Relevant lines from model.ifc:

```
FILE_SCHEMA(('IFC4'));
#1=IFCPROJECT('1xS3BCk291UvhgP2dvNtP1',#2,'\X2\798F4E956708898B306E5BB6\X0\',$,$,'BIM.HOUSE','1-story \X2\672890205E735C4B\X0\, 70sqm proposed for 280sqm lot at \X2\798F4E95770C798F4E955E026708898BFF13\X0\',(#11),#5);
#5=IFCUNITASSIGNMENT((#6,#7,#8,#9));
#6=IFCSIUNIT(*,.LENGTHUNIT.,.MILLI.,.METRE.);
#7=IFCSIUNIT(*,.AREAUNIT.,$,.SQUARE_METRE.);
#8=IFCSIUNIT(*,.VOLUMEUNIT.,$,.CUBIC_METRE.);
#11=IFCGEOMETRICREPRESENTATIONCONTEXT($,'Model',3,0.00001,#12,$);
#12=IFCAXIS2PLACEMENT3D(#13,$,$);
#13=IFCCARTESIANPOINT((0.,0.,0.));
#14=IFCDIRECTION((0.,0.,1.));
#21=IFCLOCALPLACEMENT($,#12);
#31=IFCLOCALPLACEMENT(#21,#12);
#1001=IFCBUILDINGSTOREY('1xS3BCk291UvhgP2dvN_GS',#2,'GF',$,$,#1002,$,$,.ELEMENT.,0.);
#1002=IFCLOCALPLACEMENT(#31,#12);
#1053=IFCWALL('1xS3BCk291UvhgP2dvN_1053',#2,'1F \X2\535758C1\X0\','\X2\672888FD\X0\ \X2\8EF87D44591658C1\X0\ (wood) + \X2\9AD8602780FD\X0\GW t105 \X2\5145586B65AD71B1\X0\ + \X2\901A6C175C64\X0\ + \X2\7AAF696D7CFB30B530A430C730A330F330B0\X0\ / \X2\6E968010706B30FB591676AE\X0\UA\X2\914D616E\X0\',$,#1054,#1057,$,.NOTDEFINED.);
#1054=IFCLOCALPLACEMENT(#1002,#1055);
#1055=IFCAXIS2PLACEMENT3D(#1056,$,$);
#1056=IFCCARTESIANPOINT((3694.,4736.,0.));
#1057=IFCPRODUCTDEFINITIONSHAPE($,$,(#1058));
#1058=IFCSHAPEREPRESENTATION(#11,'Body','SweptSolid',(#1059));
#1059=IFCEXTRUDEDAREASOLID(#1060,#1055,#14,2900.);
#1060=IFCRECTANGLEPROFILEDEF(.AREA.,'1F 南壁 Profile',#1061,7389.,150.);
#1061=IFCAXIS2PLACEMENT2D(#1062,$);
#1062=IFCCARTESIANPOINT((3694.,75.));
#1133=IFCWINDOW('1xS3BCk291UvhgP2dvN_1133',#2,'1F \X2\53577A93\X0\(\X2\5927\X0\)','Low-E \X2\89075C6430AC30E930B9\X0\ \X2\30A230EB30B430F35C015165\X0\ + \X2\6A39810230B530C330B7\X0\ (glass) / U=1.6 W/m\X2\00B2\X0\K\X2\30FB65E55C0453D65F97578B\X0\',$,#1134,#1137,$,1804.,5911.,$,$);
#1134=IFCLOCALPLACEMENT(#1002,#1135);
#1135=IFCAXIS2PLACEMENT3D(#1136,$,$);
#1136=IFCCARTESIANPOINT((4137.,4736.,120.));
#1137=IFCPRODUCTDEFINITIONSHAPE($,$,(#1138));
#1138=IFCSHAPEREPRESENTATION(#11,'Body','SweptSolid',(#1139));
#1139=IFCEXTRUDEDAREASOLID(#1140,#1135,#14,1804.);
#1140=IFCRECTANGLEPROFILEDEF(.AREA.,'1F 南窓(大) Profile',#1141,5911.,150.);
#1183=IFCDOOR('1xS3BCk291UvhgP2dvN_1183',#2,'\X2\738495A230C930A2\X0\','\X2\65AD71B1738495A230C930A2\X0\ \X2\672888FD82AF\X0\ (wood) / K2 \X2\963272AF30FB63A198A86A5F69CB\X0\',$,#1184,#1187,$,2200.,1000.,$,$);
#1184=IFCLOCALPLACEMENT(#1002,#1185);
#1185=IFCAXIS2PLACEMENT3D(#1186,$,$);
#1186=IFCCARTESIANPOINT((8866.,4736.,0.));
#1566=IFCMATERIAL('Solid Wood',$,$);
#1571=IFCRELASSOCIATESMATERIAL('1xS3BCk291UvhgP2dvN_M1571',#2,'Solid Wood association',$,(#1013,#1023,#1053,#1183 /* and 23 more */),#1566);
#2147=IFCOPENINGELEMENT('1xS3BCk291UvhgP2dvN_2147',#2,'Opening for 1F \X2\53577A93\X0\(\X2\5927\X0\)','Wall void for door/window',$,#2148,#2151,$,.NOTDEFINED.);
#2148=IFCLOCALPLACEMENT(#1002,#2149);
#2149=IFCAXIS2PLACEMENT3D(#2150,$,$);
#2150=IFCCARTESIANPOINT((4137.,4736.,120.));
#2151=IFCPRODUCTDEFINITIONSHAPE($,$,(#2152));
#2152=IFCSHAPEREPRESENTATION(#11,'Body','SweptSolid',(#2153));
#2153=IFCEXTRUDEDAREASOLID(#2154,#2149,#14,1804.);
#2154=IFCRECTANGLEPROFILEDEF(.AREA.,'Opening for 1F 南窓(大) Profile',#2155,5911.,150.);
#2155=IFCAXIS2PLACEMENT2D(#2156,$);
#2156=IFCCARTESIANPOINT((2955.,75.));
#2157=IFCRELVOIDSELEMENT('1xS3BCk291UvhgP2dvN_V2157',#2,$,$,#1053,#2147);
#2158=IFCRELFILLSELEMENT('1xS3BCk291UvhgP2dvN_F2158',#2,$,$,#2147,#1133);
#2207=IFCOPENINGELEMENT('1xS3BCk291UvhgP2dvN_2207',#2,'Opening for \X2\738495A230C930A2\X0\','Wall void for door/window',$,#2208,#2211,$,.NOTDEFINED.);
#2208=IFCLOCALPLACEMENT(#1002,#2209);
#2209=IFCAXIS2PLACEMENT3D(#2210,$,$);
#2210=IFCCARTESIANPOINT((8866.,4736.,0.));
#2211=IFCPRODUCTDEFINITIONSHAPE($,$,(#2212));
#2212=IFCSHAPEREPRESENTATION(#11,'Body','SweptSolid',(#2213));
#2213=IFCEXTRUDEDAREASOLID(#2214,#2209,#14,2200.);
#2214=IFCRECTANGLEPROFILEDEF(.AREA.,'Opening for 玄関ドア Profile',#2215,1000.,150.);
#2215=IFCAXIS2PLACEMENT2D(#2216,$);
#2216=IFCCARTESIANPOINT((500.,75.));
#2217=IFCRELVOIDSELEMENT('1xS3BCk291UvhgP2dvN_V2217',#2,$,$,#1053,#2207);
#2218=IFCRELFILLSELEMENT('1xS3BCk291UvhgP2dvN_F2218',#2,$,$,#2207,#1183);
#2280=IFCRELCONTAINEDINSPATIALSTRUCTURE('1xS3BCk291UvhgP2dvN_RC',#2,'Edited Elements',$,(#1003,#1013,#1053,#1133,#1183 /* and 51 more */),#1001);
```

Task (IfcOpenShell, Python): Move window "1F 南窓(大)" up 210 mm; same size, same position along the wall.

```python
import numpy as np
import ifcopenshell
import ifcopenshell.api.geometry
import ifcopenshell.util.placement
import ifcopenshell.util.unit

model = ifcopenshell.open("model.ifc")
unit_scale = ifcopenshell.util.unit.calculate_unit_scale(model)

window = model.by_id(1133)
opening = window.FillsVoids[0].RelatingOpeningElement
dz = 210.0

shift = np.array([0.0, 0.0, dz])
# The window is not placed relative to its opening, so move both.
for product in (opening, window):
    matrix = ifcopenshell.util.placement.get_local_placement(product.ObjectPlacement)
    matrix[:3, 3] += shift
    ifcopenshell.api.geometry.edit_object_placement(model, product=product, matrix=matrix, is_si=False)

print(f"moved by {dz * unit_scale:+.3f} m")

model.write("model-out.ifc")
```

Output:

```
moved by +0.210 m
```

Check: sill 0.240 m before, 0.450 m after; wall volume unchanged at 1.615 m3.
